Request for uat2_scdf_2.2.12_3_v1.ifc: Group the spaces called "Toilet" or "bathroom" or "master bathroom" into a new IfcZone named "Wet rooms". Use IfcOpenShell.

First a look at what the model holds.

```python
import ifcopenshell

model = ifcopenshell.open("uat2_scdf_2.2.12_3_v1.ifc")
print(model.schema)
seen = {}
for space in model.by_type("IfcSpace"):
    seen[space.LongName] = seen.get(space.LongName, 0) + 1
for name, count in sorted(seen.items(), key=str):
    print(count, "x", name)
print("zones:", [z.Name for z in model.by_type("IfcZone")][:20])
```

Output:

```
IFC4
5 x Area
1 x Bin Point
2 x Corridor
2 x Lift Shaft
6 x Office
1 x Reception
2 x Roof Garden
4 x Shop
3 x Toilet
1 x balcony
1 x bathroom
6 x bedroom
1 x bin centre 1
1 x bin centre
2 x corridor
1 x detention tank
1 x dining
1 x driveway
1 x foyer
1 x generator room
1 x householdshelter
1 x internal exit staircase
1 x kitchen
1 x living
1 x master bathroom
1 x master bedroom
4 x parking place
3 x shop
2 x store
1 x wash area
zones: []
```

```python
import ifcopenshell
import ifcopenshell.api.group
import ifcopenshell.api.root

model = ifcopenshell.open("uat2_scdf_2.2.12_3_v1.ifc")

names = {"Toilet", "bathroom", "master bathroom"}
spaces = [s for s in model.by_type("IfcSpace") if s.LongName in names]

zone = ifcopenshell.api.root.create_entity(model, ifc_class="IfcZone", name="Wet rooms")
ifcopenshell.api.group.assign_group(model, products=spaces, group=zone)
print(len(spaces), "spaces in", zone.Name)

model.write("uat2_scdf_2.2.12_3_v1-out.ifc")
```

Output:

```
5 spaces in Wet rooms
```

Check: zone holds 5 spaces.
